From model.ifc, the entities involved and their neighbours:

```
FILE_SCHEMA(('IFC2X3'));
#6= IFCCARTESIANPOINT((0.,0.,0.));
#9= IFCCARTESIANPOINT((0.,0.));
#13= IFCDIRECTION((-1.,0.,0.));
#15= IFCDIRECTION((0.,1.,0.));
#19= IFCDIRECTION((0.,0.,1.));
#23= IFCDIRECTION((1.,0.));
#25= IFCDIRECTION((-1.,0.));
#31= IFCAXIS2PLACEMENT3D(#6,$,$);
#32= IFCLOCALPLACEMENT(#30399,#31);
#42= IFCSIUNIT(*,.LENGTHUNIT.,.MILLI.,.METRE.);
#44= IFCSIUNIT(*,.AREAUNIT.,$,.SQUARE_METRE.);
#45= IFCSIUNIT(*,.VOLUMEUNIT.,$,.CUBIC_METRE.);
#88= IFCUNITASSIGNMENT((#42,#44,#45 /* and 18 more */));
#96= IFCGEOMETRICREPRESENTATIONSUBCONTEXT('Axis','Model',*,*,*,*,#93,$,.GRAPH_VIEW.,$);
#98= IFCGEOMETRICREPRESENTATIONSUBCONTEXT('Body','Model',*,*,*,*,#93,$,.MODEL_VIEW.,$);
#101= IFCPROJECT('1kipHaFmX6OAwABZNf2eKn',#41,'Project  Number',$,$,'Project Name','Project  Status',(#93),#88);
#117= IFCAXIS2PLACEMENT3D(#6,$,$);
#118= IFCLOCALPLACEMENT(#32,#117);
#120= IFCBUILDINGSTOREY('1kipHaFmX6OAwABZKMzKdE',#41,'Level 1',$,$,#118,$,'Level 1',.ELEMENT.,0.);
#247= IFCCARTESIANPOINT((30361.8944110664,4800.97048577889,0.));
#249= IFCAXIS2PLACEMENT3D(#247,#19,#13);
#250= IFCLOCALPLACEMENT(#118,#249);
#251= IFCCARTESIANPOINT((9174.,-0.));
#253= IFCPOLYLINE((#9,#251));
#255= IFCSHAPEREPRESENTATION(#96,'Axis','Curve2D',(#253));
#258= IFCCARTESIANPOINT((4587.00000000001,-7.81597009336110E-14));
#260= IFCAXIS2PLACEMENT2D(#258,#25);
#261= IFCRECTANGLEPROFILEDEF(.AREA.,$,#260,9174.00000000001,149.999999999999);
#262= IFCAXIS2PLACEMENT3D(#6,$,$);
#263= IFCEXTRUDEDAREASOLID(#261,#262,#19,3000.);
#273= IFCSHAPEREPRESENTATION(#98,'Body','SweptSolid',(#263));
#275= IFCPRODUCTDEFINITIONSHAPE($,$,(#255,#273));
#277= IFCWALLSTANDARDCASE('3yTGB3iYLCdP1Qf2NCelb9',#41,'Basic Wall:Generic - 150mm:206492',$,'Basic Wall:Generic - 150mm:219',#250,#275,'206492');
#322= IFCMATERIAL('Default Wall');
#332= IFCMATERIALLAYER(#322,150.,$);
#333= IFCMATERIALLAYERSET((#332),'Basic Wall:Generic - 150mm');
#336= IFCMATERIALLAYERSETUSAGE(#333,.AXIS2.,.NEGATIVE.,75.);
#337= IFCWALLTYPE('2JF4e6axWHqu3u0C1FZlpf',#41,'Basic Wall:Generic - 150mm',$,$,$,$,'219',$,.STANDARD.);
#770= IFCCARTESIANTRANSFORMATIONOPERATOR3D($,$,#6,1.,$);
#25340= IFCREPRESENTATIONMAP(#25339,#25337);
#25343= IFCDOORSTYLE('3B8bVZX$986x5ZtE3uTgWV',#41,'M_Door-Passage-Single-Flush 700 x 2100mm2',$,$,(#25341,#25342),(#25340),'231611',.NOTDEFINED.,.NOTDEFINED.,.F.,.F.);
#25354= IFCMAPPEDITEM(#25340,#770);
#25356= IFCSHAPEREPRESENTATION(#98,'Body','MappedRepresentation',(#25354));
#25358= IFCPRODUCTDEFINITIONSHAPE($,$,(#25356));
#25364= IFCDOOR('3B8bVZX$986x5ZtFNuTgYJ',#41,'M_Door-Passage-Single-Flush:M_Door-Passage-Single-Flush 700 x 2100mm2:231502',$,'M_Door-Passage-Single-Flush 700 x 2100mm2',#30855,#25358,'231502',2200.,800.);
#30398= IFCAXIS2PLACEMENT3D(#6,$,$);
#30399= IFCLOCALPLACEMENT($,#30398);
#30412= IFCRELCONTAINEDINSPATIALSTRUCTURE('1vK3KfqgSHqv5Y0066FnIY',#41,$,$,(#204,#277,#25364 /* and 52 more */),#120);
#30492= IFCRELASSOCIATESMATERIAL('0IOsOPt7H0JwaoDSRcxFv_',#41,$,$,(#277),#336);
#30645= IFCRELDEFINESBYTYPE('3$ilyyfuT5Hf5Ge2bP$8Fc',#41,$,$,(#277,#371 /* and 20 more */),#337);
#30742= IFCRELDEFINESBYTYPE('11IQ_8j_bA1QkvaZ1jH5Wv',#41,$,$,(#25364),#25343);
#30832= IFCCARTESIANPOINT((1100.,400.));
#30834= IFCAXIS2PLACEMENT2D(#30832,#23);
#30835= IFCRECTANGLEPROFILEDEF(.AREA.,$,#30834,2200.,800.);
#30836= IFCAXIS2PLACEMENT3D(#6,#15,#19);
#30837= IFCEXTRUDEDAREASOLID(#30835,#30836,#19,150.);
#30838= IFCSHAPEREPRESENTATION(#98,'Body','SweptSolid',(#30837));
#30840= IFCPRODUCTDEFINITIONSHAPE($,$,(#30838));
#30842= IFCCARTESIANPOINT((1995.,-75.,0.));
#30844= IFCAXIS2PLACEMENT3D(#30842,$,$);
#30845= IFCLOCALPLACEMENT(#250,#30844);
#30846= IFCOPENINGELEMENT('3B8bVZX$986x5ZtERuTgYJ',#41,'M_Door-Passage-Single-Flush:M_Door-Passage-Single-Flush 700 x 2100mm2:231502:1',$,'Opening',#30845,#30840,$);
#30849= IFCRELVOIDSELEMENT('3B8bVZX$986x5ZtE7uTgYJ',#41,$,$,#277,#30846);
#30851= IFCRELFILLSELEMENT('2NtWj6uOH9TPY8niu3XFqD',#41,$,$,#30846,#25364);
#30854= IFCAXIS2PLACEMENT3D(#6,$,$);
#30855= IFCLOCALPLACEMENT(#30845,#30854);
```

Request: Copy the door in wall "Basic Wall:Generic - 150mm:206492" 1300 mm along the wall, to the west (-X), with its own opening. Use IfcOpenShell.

```python
import ifcopenshell
import ifcopenshell.api.feature
import ifcopenshell.api.geometry
import ifcopenshell.api.root
import ifcopenshell.geom
import ifcopenshell.util.element
import ifcopenshell.util.placement
import ifcopenshell.util.shape
import ifcopenshell.util.unit

model = ifcopenshell.open("model.ifc")
unit_scale = ifcopenshell.util.unit.calculate_unit_scale(model)
settings = ifcopenshell.geom.settings()


def volume(element):
    """Net volume in cubic metres, openings subtracted."""
    shape = ifcopenshell.geom.create_shape(settings, element)
    return ifcopenshell.util.shape.get_volume(shape.geometry)


def reuse_history(source, copy):
    """copy_class also copies each property set's owner history, people and application; keep the originals."""
    for rel in copy.IsDefinedBy:
        if rel.is_a("IfcRelDefinesByProperties") and (history := rel.RelatingPropertyDefinition.OwnerHistory):
            rel.RelatingPropertyDefinition.OwnerHistory = source.OwnerHistory
            ifcopenshell.util.element.remove_deep2(model, history)


door = model.by_guid("3B8bVZX$986x5ZtFNuTgYJ")
opening = door.FillsVoids[0].RelatingOpeningElement
wall = opening.VoidsElements[0].RelatingBuildingElement
before = volume(wall)
shift = ifcopenshell.util.placement.get_local_placement(wall.ObjectPlacement)[:3, 0] * 1.3 / unit_scale

# copy_class copies the void relationship, type, container and properties, but no geometry.
new_opening = ifcopenshell.api.root.copy_class(model, product=opening)
new_opening.Representation = ifcopenshell.util.element.copy_deep(
    model, opening.Representation, exclude=["IfcGeometricRepresentationContext", "IfcRepresentationMap"]
)
new_opening.Name = "M_Door-Passage-Single-Flush:M_Door-Passage-Single-Flush 700 x 2100mm2"
new_door = ifcopenshell.api.root.copy_class(model, product=door)
new_door.Representation = ifcopenshell.util.element.copy_deep(
    model, door.Representation, exclude=["IfcGeometricRepresentationContext", "IfcRepresentationMap"]
)
new_door.Name = "M_Door-Passage-Single-Flush:M_Door-Passage-Single-Flush 700 x 2100mm2"
new_door.Tag = None
reuse_history(door, new_door)
fills = ifcopenshell.api.feature.add_filling(model, opening=new_opening, element=new_door)
fills.OwnerHistory = new_door.OwnerHistory  # required in IFC2X3

for old, new in ((opening, new_opening), (door, new_door)):
    matrix = ifcopenshell.util.placement.get_local_placement(old.ObjectPlacement)
    matrix[:3, 3] += shift
    ifcopenshell.api.geometry.edit_object_placement(model, product=new, matrix=matrix, is_si=False)

after = volume(wall)

print(f"wall volume {before:.3f} -> {after:.3f} m3")

model.write("model_updated.ifc")
```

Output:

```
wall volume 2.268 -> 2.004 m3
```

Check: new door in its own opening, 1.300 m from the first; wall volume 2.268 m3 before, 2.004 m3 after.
